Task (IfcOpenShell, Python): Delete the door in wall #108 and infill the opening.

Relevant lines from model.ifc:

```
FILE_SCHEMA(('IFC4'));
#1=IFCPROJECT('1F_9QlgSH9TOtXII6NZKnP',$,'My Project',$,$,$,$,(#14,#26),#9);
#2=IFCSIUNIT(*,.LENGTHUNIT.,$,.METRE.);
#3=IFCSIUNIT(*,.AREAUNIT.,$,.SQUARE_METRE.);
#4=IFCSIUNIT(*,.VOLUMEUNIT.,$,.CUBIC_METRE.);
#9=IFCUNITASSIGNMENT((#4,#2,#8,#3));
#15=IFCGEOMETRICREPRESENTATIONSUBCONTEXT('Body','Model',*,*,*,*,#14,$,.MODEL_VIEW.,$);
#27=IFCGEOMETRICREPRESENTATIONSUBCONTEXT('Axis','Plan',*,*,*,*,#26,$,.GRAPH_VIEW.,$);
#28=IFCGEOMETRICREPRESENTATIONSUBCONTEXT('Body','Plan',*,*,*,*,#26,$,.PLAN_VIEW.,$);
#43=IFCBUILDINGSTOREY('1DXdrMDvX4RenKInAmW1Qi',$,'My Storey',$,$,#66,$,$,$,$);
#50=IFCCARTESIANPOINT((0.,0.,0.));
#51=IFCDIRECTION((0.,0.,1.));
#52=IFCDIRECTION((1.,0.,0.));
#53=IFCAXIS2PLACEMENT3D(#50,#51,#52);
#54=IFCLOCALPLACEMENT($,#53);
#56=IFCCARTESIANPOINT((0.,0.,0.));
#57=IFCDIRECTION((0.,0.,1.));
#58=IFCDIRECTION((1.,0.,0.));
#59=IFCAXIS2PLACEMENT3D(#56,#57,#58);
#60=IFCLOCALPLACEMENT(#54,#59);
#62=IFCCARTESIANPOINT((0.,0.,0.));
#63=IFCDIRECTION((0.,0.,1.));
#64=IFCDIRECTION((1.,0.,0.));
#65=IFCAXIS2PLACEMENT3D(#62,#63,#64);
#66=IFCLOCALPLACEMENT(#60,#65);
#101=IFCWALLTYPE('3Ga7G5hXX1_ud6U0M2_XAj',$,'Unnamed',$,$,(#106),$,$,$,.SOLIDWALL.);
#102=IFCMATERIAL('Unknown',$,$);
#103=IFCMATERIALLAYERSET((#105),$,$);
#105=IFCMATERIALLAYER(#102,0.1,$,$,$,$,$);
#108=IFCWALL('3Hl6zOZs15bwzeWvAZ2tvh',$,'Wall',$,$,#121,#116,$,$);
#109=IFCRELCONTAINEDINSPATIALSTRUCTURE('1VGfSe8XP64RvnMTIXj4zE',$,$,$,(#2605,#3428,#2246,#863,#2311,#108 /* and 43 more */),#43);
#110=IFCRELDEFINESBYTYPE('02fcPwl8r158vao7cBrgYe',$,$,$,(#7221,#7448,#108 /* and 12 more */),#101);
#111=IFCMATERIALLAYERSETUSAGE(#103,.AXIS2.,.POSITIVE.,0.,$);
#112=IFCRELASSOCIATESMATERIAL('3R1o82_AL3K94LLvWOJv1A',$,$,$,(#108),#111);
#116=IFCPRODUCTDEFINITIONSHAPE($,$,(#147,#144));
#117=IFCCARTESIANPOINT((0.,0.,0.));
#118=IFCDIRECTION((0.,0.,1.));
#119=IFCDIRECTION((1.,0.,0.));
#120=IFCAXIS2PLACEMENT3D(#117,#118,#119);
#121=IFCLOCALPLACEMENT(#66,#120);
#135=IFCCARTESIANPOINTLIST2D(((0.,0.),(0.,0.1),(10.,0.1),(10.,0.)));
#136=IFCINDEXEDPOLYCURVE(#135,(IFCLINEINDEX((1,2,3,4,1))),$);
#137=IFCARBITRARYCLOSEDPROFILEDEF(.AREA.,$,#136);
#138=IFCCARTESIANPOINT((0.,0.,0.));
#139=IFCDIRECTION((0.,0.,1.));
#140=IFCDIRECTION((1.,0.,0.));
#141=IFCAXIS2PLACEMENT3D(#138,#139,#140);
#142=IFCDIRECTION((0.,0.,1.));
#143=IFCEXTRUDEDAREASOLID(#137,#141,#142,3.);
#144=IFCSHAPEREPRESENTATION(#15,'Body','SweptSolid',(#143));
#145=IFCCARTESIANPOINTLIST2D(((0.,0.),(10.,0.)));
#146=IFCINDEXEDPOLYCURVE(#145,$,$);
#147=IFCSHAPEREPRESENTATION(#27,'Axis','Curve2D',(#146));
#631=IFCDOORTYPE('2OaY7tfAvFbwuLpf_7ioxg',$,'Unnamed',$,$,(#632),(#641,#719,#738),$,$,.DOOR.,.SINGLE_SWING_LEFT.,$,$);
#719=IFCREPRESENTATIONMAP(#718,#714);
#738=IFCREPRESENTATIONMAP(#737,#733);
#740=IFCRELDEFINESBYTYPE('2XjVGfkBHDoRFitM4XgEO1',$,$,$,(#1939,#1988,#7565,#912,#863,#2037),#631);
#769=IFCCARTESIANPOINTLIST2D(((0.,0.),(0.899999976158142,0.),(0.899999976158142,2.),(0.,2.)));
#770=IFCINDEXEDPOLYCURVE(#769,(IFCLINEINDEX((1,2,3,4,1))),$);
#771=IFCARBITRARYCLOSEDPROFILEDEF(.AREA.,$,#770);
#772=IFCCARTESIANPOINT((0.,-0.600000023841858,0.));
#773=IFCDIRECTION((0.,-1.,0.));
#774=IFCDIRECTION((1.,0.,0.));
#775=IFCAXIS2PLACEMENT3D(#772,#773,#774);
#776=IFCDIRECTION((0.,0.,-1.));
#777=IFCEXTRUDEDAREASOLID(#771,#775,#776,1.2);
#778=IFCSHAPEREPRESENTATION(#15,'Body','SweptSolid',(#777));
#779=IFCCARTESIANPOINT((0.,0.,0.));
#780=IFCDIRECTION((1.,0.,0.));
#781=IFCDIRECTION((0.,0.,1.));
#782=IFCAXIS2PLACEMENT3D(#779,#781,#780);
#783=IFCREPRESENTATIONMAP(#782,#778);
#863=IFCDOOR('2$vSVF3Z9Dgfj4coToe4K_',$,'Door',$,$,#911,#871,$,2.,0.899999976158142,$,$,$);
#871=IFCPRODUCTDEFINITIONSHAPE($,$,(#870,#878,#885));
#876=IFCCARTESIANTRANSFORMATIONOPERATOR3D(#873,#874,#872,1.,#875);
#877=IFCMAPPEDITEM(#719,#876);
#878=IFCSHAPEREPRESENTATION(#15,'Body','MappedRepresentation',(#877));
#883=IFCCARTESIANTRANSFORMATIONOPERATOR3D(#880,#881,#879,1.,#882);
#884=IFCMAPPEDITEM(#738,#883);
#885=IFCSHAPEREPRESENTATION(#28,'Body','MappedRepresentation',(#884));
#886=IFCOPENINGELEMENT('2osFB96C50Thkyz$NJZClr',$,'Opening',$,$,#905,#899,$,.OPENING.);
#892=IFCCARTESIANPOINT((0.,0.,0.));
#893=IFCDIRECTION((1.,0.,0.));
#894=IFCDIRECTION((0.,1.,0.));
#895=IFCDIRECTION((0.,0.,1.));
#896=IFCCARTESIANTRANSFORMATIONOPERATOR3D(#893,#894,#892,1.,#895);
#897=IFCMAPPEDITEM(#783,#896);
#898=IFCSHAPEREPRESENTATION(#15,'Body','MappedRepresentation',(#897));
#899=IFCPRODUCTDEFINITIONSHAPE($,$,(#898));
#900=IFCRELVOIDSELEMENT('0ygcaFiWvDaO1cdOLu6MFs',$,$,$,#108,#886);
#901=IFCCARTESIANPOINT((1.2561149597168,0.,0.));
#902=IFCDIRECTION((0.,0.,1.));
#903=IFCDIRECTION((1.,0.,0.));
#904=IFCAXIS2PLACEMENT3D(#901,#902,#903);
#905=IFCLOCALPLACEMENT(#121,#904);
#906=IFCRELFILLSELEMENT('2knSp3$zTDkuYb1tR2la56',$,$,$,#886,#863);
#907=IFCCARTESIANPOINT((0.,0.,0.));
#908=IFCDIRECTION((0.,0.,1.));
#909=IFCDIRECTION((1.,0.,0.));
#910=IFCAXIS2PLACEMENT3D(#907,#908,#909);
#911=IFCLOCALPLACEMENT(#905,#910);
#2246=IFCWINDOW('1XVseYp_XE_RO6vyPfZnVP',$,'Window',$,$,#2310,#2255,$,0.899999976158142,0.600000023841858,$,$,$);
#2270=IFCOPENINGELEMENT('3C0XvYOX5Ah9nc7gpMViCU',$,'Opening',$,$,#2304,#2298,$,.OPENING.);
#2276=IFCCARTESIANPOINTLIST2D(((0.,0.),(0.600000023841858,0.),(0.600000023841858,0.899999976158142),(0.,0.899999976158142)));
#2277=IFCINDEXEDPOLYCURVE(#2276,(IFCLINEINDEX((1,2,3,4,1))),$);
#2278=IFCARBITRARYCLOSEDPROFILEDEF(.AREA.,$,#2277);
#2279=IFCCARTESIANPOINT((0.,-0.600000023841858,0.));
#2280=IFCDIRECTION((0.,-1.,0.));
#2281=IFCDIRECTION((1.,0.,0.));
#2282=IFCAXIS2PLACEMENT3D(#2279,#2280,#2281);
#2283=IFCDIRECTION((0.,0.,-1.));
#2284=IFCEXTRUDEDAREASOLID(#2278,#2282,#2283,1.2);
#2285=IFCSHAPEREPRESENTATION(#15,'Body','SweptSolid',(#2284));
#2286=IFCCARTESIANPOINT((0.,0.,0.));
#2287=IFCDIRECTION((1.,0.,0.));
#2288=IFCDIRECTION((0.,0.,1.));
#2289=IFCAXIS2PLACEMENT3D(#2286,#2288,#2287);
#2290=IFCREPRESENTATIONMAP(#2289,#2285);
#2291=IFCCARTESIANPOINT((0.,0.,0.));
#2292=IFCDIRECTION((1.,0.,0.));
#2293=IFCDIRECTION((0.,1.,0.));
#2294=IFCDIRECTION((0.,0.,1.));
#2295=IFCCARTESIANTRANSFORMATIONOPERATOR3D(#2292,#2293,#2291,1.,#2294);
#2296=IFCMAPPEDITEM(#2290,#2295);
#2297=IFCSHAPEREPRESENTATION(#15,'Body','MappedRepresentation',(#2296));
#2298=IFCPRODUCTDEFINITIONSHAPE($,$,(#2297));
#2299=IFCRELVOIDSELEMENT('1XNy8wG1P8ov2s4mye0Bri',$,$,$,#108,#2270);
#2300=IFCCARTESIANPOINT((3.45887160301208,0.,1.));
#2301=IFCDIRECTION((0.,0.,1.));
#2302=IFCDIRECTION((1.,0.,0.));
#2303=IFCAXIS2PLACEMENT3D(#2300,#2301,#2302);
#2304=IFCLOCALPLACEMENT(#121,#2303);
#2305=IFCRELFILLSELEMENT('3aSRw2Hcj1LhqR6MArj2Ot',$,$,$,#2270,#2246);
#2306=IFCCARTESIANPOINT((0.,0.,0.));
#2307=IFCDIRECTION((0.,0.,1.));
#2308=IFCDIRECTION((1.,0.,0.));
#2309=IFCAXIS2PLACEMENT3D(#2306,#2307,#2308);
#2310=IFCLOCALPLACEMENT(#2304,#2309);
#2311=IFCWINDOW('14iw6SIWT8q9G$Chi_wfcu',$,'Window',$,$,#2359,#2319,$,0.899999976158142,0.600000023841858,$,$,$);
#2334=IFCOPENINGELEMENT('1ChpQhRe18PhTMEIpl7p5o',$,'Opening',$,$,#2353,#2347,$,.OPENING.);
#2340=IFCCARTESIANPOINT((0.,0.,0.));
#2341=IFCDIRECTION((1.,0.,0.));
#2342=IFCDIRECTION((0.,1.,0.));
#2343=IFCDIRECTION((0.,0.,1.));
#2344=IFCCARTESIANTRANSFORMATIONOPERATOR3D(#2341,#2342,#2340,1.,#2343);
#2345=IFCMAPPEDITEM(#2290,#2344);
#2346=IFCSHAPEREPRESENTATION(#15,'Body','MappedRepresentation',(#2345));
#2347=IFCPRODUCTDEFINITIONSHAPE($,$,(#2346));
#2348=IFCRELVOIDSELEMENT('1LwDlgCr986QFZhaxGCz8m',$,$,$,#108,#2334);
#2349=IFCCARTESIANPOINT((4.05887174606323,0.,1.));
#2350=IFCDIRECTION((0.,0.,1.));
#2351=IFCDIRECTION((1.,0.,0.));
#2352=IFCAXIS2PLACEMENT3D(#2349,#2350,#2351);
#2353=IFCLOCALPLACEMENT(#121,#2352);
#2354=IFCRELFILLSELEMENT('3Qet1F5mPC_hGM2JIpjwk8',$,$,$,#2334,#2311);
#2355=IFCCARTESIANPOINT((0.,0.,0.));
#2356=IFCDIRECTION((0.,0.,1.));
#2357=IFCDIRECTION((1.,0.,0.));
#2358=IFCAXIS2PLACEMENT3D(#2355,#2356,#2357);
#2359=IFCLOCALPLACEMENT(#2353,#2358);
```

```python
import ifcopenshell
import ifcopenshell.api.feature
import ifcopenshell.api.root
import ifcopenshell.geom
import ifcopenshell.util.shape

model = ifcopenshell.open("model.ifc")
settings = ifcopenshell.geom.settings()


def volume(element):
    """Net volume in cubic metres, openings subtracted."""
    shape = ifcopenshell.geom.create_shape(settings, element)
    return ifcopenshell.util.shape.get_volume(shape.geometry)


door = model.by_id(863)
opening = door.FillsVoids[0].RelatingOpeningElement
wall = opening.VoidsElements[0].RelatingBuildingElement
before = volume(wall)

ifcopenshell.api.root.remove_product(model, product=door)
ifcopenshell.api.feature.remove_feature(model, feature=opening)

after = volume(wall)

print(f"wall volume {before:.3f} -> {after:.3f} m3")

model.write("model_rev.ifc")
```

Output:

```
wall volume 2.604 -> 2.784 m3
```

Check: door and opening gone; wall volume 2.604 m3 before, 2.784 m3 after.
